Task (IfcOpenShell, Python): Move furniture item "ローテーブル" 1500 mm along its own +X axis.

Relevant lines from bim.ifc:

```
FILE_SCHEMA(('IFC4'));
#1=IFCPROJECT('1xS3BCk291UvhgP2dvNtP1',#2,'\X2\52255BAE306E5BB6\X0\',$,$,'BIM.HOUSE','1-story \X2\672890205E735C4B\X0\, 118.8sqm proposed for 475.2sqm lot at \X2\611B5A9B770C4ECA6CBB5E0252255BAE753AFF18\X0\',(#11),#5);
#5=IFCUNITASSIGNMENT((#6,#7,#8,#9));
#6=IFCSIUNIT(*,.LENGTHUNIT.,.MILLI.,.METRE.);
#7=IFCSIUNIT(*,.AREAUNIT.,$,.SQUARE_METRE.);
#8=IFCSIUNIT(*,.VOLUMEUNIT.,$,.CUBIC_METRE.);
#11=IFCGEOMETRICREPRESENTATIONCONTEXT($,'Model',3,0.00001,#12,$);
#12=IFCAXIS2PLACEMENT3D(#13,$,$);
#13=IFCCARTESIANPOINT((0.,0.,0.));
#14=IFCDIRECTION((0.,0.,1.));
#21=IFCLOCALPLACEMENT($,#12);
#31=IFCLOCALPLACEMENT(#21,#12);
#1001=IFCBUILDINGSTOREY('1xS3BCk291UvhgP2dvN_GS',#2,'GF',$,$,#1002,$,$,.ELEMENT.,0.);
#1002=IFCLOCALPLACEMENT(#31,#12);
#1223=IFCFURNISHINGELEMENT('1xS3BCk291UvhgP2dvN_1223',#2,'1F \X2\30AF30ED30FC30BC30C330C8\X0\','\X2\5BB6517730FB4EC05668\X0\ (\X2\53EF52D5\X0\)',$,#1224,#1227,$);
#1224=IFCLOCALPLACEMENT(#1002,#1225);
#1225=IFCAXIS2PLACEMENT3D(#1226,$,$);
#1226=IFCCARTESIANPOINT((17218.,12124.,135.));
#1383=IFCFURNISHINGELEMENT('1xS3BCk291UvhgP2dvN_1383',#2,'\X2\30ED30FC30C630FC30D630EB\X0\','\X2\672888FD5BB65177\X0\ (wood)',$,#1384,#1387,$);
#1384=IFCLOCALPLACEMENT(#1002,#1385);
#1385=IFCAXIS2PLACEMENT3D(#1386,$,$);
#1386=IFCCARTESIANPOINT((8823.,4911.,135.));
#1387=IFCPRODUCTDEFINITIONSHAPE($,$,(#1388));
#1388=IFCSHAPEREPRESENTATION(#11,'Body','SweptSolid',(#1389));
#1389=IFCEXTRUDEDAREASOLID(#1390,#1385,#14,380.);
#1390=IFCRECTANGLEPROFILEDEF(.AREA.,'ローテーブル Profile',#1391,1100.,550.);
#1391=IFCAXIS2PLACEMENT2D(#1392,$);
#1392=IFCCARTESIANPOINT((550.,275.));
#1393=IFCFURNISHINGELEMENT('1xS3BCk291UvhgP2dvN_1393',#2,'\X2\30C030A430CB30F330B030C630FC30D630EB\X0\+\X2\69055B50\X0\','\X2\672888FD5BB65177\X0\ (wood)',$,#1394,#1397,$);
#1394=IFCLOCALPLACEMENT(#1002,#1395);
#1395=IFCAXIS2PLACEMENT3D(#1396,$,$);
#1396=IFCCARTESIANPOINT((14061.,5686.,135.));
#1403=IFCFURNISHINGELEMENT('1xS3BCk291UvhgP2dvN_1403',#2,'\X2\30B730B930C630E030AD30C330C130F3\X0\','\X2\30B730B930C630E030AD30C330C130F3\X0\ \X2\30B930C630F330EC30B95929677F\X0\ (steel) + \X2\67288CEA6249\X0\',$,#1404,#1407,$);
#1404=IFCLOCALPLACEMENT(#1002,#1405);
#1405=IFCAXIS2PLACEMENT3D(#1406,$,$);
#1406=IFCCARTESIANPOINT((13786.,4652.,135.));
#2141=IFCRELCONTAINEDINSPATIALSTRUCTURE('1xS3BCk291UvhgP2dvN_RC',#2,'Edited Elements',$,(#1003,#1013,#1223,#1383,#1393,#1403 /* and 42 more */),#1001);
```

```python
import ifcopenshell
import ifcopenshell.api.geometry
import ifcopenshell.util.placement

model = ifcopenshell.open("bim.ifc")

item = model.by_id(1383)
matrix = ifcopenshell.util.placement.get_local_placement(item.ObjectPlacement)
matrix[:3, 3] += matrix[:3, 0] * 1500.0
ifcopenshell.api.geometry.edit_object_placement(model, product=item, matrix=matrix, is_si=False)

print(ifcopenshell.util.placement.get_local_placement(item.ObjectPlacement).round(3) + 0.0)

model.write("bim_rev.ifc")
```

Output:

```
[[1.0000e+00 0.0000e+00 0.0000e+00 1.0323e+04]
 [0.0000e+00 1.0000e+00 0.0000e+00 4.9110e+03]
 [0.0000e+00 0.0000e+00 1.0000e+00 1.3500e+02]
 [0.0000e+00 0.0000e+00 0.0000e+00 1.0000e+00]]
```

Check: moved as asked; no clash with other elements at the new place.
